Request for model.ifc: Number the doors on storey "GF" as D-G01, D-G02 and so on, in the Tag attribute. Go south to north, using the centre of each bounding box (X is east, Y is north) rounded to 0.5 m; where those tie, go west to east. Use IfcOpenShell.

First a look at what the model holds.

```python
import ifcopenshell
import ifcopenshell.util.element
import ifcopenshell.util.placement

model = ifcopenshell.open("model.ifc")
print(model.schema)
storey = next(s for s in model.by_type("IfcBuildingStorey") if s.Name == "GF")
doors = [e for e in ifcopenshell.util.element.get_decomposition(storey) if e.is_a("IfcDoor")]
for e in sorted(doors, key=lambda e: e.id()):
    origin = ifcopenshell.util.placement.get_local_placement(e.ObjectPlacement)[:3, 3]
    print(e.id(), e.Tag, e.Name, origin.round(2) + 0.0, sep=" | ")
```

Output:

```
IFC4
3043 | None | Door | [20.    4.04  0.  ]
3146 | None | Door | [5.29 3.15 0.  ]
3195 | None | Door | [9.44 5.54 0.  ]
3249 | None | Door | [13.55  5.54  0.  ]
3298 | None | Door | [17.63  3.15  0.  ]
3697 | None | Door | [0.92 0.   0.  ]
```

```python
import ifcopenshell
import ifcopenshell.geom
import ifcopenshell.util.element
import ifcopenshell.util.shape

model = ifcopenshell.open("model.ifc")
settings = ifcopenshell.geom.settings()
settings.set("use-world-coords", True)


def centre(element):
    shape = ifcopenshell.geom.create_shape(settings, element)
    return ifcopenshell.util.shape.get_bbox_centroid(shape.geometry)


storey = next(s for s in model.by_type("IfcBuildingStorey") if s.Name == "GF")
doors = [e for e in ifcopenshell.util.element.get_decomposition(storey) if e.is_a("IfcDoor")]

# Insertion points can sit at a corner or the storey origin, so sort by the geometry (in metres).
centres = {e: centre(e) for e in doors}
doors.sort(key=lambda e: (round(centres[e][1] / 0.5), centres[e][0]))

for i, e in enumerate(doors, start=1):
    number = f"D-G{i:02d}"
    e.Tag = number
    print(e.id(), number)

model.write("model_rev.ifc")
```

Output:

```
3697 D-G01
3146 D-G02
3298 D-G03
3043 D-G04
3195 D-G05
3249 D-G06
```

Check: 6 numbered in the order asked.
